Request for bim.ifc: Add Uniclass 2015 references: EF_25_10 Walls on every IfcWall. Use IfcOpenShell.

First a look at what the model holds.

```python
import ifcopenshell

model = ifcopenshell.open("bim.ifc")
print(model.schema)
print("classifications:", [c.Name for c in model.by_type("IfcClassification")])
for ifc_class in ("IfcDoor", "IfcRoof", "IfcStair", "IfcWall", "IfcWindow"):
    print(ifc_class, len(model.by_type(ifc_class)))
```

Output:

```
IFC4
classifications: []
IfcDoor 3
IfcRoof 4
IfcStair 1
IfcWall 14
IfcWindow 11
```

```python
import ifcopenshell
import ifcopenshell.api.classification

model = ifcopenshell.open("bim.ifc")

system = ifcopenshell.api.classification.add_classification(model, classification="Uniclass 2015")

codes = {
    "IfcWall": ("EF_25_10", "Walls"),
}
for ifc_class, (code, name) in codes.items():
    products = model.by_type(ifc_class)
    ifcopenshell.api.classification.add_reference(
        model, products=products, classification=system, identification=code, name=name
    )
    print(code, len(products))

model.write("bim_updated.ifc")
```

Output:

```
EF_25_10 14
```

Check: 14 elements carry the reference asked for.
